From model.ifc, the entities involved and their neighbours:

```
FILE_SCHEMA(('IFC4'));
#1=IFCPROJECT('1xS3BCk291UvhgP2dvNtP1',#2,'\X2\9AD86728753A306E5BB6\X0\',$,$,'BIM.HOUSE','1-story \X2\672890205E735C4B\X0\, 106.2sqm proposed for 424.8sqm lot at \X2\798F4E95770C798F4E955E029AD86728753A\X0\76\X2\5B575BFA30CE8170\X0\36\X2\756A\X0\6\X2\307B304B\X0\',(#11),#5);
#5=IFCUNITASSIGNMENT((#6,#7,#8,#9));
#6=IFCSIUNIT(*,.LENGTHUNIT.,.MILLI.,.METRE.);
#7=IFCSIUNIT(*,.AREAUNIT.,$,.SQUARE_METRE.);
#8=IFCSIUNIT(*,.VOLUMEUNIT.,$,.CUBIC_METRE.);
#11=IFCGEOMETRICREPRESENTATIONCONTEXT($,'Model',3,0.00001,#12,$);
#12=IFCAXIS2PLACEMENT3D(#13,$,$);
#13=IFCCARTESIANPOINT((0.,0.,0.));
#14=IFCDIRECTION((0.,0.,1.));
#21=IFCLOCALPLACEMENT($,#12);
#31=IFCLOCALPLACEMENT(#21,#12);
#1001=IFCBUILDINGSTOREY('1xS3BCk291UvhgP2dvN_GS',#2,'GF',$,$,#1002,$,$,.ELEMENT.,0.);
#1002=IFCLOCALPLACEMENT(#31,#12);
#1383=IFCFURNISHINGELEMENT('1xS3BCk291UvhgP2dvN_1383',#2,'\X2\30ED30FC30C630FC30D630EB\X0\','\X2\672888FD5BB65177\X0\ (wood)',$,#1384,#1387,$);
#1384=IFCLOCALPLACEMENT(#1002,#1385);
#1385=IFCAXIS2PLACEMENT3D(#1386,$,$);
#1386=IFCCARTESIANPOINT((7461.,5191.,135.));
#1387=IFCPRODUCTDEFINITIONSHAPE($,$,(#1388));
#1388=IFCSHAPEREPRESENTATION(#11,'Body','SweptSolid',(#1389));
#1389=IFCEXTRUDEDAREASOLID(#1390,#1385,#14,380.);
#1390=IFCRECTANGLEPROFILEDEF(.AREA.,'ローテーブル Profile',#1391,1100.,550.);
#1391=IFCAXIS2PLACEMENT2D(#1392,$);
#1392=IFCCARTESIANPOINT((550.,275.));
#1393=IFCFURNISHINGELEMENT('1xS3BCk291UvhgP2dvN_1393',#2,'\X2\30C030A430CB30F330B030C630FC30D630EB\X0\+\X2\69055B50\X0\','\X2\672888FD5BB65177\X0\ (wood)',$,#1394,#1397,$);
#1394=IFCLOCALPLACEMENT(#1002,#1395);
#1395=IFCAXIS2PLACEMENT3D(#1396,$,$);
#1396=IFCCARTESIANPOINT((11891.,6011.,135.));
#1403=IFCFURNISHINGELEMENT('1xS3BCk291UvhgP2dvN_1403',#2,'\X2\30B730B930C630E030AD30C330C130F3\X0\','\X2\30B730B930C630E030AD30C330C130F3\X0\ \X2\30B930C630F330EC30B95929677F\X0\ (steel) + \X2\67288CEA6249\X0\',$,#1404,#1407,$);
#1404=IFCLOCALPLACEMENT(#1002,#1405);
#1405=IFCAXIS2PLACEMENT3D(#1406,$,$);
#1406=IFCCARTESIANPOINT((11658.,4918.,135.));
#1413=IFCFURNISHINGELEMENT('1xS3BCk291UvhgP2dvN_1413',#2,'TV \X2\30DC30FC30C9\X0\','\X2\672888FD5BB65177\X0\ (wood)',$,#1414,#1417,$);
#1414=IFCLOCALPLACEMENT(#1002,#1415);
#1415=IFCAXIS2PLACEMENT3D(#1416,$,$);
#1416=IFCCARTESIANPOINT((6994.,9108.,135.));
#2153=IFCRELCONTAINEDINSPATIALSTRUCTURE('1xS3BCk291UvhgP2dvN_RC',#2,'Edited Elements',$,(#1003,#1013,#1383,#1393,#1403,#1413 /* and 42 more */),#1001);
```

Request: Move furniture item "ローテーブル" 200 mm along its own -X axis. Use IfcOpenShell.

```python
import ifcopenshell
import ifcopenshell.api.geometry
import ifcopenshell.util.placement
import ifcopenshell.util.unit

model = ifcopenshell.open("model.ifc")
unit_scale = ifcopenshell.util.unit.calculate_unit_scale(model)

item = model.by_guid("1xS3BCk291UvhgP2dvN_1383")
matrix = ifcopenshell.util.placement.get_local_placement(item.ObjectPlacement)
matrix[:3, 3] -= matrix[:3, 0] * 0.2 / unit_scale
ifcopenshell.api.geometry.edit_object_placement(model, product=item, matrix=matrix, is_si=False)

print(ifcopenshell.util.placement.get_local_placement(item.ObjectPlacement).round(3) + 0.0)

model.write("model_updated.ifc")
```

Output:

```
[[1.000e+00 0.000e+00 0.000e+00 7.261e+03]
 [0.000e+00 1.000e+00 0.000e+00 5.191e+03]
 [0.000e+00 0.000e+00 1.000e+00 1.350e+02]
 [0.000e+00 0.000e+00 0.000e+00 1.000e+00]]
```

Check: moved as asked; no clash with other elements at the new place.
